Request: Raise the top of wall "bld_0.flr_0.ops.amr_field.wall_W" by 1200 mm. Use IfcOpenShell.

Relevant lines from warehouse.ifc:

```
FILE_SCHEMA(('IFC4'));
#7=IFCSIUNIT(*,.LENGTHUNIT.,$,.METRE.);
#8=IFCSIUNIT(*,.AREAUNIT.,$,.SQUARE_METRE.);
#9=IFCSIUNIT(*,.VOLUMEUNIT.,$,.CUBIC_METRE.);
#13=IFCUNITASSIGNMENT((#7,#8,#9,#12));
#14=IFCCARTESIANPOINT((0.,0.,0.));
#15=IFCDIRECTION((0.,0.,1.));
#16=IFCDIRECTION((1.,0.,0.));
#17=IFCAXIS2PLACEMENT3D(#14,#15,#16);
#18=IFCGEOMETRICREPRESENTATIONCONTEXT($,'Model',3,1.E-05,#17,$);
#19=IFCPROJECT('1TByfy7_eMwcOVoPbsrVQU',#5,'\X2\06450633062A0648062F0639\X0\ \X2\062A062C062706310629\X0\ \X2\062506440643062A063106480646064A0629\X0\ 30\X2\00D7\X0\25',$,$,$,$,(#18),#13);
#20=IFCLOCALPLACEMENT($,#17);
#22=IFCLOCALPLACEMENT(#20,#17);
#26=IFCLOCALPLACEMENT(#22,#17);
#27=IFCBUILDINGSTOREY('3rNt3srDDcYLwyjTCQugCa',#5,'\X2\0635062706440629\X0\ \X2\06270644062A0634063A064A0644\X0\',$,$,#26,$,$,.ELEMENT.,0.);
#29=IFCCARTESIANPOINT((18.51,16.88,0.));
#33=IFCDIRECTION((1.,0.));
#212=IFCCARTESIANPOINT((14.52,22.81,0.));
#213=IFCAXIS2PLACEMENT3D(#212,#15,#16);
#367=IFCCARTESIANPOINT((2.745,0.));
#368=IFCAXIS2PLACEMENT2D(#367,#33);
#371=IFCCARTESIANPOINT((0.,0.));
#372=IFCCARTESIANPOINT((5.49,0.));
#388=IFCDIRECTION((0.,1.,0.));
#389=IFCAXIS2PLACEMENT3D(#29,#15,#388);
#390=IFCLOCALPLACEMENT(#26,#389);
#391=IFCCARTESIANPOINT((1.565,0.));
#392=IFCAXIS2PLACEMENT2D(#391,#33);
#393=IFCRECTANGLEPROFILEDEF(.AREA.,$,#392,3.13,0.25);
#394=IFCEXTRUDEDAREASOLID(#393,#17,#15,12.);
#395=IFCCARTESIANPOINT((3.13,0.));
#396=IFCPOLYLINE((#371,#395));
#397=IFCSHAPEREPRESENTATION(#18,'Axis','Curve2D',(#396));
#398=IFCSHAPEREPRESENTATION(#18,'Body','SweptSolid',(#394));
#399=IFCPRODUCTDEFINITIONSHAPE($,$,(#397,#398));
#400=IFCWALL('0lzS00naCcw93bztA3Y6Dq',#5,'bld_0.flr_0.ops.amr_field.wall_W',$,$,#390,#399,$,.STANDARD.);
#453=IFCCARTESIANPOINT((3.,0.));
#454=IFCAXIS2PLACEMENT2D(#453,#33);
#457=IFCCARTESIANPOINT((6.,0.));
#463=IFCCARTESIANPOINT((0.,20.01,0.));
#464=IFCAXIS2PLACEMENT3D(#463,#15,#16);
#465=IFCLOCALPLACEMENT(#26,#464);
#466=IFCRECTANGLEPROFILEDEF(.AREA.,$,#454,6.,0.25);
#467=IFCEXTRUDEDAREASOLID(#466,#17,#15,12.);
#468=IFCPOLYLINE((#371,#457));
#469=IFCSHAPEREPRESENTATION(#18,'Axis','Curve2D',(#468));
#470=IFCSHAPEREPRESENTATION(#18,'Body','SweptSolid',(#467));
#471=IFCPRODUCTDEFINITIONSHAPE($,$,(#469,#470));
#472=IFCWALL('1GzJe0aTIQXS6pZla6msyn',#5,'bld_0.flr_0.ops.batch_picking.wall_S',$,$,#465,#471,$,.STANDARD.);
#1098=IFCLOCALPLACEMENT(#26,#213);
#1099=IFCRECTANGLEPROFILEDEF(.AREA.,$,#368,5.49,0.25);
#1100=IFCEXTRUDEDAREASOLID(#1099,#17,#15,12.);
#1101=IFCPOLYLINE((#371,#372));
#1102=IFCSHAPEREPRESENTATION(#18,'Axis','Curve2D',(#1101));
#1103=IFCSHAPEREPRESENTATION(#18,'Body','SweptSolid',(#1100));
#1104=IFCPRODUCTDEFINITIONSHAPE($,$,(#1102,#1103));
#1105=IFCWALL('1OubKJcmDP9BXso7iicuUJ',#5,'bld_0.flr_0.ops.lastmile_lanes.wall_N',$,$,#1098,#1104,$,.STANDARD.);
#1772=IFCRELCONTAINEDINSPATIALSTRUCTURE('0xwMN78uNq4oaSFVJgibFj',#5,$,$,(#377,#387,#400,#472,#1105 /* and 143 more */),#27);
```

```python
import ifcopenshell
import ifcopenshell.geom
import ifcopenshell.util.shape
import ifcopenshell.util.unit

model = ifcopenshell.open("warehouse.ifc")
unit_scale = ifcopenshell.util.unit.calculate_unit_scale(model)
settings = ifcopenshell.geom.settings()


def volume(element):
    """Net volume in cubic metres, openings subtracted."""
    shape = ifcopenshell.geom.create_shape(settings, element)
    return ifcopenshell.util.shape.get_volume(shape.geometry)


wall = model.by_id(400)
before = volume(wall)

body = next(r for r in wall.Representation.Representations if r.RepresentationIdentifier == "Body")
solid = body.Items[0]
old_height = solid.Depth
solid.Depth += 1.2 / unit_scale
after = volume(wall)

print(f"height {old_height:g} -> {solid.Depth:g}, volume {before:.3f} -> {after:.3f} m3")

model.write("warehouse_updated.ifc")
```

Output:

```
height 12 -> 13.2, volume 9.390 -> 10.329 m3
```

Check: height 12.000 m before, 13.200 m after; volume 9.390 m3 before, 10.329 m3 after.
